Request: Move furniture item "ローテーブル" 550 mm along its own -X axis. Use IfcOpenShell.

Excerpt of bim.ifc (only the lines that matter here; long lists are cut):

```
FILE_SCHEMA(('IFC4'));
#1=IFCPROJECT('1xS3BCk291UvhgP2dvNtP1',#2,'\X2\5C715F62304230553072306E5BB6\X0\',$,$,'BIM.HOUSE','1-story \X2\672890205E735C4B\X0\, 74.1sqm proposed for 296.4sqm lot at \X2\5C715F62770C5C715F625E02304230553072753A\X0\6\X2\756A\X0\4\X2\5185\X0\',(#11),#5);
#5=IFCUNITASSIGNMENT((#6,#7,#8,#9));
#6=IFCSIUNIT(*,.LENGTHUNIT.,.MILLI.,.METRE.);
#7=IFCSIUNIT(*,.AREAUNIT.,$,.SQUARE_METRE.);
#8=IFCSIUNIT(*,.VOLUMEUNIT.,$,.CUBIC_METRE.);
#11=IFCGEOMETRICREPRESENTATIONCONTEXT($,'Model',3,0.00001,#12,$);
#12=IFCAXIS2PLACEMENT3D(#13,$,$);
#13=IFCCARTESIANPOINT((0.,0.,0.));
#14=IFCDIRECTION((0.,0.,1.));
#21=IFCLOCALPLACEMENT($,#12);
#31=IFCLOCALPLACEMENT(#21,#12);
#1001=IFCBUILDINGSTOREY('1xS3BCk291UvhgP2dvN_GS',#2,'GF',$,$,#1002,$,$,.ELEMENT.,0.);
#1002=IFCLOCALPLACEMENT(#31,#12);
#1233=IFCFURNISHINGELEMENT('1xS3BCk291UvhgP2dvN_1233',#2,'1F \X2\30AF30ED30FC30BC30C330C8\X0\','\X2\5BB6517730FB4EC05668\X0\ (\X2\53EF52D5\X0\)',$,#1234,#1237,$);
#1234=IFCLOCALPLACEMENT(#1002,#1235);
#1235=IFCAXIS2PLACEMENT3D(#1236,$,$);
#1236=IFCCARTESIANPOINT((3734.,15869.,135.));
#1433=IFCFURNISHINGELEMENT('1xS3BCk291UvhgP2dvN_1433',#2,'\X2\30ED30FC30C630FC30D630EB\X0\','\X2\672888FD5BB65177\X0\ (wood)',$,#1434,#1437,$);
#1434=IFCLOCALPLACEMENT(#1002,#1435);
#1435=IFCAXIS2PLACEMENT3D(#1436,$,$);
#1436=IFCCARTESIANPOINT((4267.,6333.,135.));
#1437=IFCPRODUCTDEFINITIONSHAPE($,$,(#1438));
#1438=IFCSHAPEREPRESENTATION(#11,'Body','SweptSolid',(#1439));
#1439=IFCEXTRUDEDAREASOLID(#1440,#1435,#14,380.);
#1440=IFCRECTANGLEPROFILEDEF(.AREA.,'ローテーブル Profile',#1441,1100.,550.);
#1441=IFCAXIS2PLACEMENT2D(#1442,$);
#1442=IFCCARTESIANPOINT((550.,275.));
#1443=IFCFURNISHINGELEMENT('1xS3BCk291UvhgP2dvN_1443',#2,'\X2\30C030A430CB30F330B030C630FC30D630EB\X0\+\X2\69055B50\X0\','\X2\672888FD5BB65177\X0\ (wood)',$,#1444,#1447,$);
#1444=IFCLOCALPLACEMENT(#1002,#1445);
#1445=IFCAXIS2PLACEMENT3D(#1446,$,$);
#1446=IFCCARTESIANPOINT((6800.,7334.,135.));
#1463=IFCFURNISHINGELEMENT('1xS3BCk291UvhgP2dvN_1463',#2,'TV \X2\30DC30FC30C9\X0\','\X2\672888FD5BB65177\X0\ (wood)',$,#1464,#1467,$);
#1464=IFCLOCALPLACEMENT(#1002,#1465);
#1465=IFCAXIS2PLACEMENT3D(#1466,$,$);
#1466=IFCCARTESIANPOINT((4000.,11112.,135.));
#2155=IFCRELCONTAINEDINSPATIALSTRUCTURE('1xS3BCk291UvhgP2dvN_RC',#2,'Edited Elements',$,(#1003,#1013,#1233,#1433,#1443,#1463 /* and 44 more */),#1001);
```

```python
import ifcopenshell
import ifcopenshell.api.geometry
import ifcopenshell.util.placement
import ifcopenshell.util.unit

model = ifcopenshell.open("bim.ifc")
unit_scale = ifcopenshell.util.unit.calculate_unit_scale(model)

item = model.by_guid("1xS3BCk291UvhgP2dvN_1433")
matrix = ifcopenshell.util.placement.get_local_placement(item.ObjectPlacement)
matrix[:3, 3] -= matrix[:3, 0] * 0.55 / unit_scale
ifcopenshell.api.geometry.edit_object_placement(model, product=item, matrix=matrix, is_si=False)

print(ifcopenshell.util.placement.get_local_placement(item.ObjectPlacement).round(3) + 0.0)

model.write("bim_v2.ifc")
```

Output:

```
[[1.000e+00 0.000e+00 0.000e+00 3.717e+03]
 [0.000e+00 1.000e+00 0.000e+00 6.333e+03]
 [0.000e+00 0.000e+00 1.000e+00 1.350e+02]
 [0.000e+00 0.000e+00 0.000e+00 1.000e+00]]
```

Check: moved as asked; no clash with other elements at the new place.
